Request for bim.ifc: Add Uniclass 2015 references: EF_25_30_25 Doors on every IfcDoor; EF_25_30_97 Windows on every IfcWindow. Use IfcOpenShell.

First a look at what the model holds.

```python
import ifcopenshell

model = ifcopenshell.open("bim.ifc")
print(model.schema)
print("classifications:", [c.Name for c in model.by_type("IfcClassification")])
for ifc_class in ("IfcDoor", "IfcRoof", "IfcStair", "IfcWall", "IfcWindow"):
    print(ifc_class, len(model.by_type(ifc_class)))
```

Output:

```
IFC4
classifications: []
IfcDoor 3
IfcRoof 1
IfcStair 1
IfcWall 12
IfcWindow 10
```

```python
import ifcopenshell
import ifcopenshell.api.classification

model = ifcopenshell.open("bim.ifc")

system = ifcopenshell.api.classification.add_classification(model, classification="Uniclass 2015")

codes = {
    "IfcDoor": ("EF_25_30_25", "Doors"),
    "IfcWindow": ("EF_25_30_97", "Windows"),
}
for ifc_class, (code, name) in codes.items():
    products = model.by_type(ifc_class)
    ifcopenshell.api.classification.add_reference(
        model, products=products, classification=system, identification=code, name=name
    )
    print(code, len(products))

model.write("bim-out.ifc")
```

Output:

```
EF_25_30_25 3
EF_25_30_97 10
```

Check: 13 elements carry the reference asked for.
